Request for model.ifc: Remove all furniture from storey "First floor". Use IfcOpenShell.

First a look at what the model holds.

```python
import ifcopenshell
import ifcopenshell.util.element

model = ifcopenshell.open("model.ifc")
print(model.schema)
storey = next(s for s in model.by_type("IfcBuildingStorey") if s.Name == "First floor")
furniture = [e for e in ifcopenshell.util.element.get_decomposition(storey) if e.is_a("IfcFurnishingElement")]
seen = {}
for e in furniture:
    element_type = ifcopenshell.util.element.get_type(e)
    name = element_type.Name if element_type not in (None, e) else None
    seen[name] = seen.get(name, 0) + 1
for name, count in sorted(seen.items(), key=str):
    print(count, "x", name)
```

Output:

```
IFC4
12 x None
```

```python
import ifcopenshell
import ifcopenshell.api.root
import ifcopenshell.util.element

model = ifcopenshell.open("model.ifc")

storey = next(s for s in model.by_type("IfcBuildingStorey") if s.Name == "First floor")
furniture = [e for e in ifcopenshell.util.element.get_decomposition(storey) if e.is_a("IfcFurnishingElement")]

for e in furniture:
    ifcopenshell.api.root.remove_product(model, product=e)
print(len(furniture), "removed")

model.write("model_v2.ifc")
```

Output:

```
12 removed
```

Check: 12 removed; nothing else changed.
